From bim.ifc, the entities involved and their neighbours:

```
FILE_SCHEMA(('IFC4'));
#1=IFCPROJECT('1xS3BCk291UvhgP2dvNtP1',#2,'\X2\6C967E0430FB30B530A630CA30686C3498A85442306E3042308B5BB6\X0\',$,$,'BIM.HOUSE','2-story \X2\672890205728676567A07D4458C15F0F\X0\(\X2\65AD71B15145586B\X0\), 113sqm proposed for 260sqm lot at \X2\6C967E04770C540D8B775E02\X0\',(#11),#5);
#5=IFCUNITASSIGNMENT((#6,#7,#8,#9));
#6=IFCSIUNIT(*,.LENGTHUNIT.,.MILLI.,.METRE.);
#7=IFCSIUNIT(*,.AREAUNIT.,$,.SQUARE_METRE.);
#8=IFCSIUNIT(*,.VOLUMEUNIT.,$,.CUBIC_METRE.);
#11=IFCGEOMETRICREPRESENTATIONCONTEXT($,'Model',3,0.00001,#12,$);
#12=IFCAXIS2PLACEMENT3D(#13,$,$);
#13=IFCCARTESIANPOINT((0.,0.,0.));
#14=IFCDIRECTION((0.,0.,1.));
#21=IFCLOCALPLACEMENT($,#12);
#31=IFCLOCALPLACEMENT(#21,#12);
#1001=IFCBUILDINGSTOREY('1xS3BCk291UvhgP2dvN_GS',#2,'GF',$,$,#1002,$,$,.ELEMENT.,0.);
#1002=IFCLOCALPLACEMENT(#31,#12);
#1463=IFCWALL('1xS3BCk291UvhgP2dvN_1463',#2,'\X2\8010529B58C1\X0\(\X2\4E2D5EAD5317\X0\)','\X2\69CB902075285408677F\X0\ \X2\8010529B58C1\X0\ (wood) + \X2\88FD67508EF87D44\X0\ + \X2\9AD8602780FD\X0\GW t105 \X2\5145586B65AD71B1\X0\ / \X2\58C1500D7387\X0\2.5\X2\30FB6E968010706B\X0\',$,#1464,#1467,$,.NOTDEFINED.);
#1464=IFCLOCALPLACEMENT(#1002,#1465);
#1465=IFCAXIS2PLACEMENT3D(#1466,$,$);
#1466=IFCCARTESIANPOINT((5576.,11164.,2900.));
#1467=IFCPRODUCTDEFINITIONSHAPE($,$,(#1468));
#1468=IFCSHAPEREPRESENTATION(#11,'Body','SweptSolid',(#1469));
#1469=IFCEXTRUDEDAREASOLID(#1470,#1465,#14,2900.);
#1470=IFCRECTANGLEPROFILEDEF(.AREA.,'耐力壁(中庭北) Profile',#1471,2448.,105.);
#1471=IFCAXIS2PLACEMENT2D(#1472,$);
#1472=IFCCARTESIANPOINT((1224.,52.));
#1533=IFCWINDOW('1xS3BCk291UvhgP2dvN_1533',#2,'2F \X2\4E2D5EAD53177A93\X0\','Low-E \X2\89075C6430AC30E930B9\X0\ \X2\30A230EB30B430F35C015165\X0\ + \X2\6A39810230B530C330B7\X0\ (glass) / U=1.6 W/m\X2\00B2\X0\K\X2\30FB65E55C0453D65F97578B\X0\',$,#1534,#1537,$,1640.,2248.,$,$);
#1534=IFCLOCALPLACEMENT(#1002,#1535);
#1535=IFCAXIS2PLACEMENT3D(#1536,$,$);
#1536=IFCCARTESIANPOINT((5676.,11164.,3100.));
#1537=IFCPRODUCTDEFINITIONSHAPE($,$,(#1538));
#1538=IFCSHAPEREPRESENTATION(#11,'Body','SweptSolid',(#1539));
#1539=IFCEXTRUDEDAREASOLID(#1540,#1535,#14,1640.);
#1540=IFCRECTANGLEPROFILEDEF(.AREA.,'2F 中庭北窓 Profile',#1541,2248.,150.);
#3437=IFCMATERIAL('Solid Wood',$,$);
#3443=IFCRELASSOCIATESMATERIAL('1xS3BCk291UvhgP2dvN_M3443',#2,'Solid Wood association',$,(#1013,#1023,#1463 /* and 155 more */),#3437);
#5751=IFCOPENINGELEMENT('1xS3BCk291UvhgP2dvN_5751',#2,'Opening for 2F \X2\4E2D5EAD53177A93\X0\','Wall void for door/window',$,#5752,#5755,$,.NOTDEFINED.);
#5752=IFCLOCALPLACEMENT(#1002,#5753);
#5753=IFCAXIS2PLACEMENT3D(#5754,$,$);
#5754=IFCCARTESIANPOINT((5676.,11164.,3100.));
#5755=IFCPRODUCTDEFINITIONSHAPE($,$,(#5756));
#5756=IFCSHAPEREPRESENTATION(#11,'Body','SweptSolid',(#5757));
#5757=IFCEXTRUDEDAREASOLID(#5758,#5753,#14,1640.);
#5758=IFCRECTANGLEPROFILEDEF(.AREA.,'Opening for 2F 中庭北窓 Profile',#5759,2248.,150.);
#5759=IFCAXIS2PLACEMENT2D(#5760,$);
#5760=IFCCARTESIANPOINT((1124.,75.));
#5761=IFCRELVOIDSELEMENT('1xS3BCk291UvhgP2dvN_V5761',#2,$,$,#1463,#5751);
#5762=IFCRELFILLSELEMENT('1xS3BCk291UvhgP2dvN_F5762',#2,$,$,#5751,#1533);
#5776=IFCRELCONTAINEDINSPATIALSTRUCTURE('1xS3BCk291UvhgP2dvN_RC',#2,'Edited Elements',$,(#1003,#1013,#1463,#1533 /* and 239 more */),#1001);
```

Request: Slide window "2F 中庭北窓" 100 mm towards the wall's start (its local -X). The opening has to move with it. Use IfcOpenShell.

```python
import ifcopenshell
import ifcopenshell.api.geometry
import ifcopenshell.util.placement

model = ifcopenshell.open("bim.ifc")

window = model.by_guid("1xS3BCk291UvhgP2dvN_1533")
opening = window.FillsVoids[0].RelatingOpeningElement
wall = opening.VoidsElements[0].RelatingBuildingElement

wall_matrix = ifcopenshell.util.placement.get_local_placement(wall.ObjectPlacement)
shift = wall_matrix[:3, 0] * -100.0
before = ifcopenshell.util.placement.get_local_placement(window.ObjectPlacement)[:3, 3].copy()

# The window is not placed relative to its opening, so move both.
for product in (opening, window):
    matrix = ifcopenshell.util.placement.get_local_placement(product.ObjectPlacement)
    matrix[:3, 3] += shift
    ifcopenshell.api.geometry.edit_object_placement(model, product=product, matrix=matrix, is_si=False)

after = ifcopenshell.util.placement.get_local_placement(window.ObjectPlacement)[:3, 3]
print("window moved by", (after - before).round(3) + 0.0)

model.write("bim_rev.ifc")
```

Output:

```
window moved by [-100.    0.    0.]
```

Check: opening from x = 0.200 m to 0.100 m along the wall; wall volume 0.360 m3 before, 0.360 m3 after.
